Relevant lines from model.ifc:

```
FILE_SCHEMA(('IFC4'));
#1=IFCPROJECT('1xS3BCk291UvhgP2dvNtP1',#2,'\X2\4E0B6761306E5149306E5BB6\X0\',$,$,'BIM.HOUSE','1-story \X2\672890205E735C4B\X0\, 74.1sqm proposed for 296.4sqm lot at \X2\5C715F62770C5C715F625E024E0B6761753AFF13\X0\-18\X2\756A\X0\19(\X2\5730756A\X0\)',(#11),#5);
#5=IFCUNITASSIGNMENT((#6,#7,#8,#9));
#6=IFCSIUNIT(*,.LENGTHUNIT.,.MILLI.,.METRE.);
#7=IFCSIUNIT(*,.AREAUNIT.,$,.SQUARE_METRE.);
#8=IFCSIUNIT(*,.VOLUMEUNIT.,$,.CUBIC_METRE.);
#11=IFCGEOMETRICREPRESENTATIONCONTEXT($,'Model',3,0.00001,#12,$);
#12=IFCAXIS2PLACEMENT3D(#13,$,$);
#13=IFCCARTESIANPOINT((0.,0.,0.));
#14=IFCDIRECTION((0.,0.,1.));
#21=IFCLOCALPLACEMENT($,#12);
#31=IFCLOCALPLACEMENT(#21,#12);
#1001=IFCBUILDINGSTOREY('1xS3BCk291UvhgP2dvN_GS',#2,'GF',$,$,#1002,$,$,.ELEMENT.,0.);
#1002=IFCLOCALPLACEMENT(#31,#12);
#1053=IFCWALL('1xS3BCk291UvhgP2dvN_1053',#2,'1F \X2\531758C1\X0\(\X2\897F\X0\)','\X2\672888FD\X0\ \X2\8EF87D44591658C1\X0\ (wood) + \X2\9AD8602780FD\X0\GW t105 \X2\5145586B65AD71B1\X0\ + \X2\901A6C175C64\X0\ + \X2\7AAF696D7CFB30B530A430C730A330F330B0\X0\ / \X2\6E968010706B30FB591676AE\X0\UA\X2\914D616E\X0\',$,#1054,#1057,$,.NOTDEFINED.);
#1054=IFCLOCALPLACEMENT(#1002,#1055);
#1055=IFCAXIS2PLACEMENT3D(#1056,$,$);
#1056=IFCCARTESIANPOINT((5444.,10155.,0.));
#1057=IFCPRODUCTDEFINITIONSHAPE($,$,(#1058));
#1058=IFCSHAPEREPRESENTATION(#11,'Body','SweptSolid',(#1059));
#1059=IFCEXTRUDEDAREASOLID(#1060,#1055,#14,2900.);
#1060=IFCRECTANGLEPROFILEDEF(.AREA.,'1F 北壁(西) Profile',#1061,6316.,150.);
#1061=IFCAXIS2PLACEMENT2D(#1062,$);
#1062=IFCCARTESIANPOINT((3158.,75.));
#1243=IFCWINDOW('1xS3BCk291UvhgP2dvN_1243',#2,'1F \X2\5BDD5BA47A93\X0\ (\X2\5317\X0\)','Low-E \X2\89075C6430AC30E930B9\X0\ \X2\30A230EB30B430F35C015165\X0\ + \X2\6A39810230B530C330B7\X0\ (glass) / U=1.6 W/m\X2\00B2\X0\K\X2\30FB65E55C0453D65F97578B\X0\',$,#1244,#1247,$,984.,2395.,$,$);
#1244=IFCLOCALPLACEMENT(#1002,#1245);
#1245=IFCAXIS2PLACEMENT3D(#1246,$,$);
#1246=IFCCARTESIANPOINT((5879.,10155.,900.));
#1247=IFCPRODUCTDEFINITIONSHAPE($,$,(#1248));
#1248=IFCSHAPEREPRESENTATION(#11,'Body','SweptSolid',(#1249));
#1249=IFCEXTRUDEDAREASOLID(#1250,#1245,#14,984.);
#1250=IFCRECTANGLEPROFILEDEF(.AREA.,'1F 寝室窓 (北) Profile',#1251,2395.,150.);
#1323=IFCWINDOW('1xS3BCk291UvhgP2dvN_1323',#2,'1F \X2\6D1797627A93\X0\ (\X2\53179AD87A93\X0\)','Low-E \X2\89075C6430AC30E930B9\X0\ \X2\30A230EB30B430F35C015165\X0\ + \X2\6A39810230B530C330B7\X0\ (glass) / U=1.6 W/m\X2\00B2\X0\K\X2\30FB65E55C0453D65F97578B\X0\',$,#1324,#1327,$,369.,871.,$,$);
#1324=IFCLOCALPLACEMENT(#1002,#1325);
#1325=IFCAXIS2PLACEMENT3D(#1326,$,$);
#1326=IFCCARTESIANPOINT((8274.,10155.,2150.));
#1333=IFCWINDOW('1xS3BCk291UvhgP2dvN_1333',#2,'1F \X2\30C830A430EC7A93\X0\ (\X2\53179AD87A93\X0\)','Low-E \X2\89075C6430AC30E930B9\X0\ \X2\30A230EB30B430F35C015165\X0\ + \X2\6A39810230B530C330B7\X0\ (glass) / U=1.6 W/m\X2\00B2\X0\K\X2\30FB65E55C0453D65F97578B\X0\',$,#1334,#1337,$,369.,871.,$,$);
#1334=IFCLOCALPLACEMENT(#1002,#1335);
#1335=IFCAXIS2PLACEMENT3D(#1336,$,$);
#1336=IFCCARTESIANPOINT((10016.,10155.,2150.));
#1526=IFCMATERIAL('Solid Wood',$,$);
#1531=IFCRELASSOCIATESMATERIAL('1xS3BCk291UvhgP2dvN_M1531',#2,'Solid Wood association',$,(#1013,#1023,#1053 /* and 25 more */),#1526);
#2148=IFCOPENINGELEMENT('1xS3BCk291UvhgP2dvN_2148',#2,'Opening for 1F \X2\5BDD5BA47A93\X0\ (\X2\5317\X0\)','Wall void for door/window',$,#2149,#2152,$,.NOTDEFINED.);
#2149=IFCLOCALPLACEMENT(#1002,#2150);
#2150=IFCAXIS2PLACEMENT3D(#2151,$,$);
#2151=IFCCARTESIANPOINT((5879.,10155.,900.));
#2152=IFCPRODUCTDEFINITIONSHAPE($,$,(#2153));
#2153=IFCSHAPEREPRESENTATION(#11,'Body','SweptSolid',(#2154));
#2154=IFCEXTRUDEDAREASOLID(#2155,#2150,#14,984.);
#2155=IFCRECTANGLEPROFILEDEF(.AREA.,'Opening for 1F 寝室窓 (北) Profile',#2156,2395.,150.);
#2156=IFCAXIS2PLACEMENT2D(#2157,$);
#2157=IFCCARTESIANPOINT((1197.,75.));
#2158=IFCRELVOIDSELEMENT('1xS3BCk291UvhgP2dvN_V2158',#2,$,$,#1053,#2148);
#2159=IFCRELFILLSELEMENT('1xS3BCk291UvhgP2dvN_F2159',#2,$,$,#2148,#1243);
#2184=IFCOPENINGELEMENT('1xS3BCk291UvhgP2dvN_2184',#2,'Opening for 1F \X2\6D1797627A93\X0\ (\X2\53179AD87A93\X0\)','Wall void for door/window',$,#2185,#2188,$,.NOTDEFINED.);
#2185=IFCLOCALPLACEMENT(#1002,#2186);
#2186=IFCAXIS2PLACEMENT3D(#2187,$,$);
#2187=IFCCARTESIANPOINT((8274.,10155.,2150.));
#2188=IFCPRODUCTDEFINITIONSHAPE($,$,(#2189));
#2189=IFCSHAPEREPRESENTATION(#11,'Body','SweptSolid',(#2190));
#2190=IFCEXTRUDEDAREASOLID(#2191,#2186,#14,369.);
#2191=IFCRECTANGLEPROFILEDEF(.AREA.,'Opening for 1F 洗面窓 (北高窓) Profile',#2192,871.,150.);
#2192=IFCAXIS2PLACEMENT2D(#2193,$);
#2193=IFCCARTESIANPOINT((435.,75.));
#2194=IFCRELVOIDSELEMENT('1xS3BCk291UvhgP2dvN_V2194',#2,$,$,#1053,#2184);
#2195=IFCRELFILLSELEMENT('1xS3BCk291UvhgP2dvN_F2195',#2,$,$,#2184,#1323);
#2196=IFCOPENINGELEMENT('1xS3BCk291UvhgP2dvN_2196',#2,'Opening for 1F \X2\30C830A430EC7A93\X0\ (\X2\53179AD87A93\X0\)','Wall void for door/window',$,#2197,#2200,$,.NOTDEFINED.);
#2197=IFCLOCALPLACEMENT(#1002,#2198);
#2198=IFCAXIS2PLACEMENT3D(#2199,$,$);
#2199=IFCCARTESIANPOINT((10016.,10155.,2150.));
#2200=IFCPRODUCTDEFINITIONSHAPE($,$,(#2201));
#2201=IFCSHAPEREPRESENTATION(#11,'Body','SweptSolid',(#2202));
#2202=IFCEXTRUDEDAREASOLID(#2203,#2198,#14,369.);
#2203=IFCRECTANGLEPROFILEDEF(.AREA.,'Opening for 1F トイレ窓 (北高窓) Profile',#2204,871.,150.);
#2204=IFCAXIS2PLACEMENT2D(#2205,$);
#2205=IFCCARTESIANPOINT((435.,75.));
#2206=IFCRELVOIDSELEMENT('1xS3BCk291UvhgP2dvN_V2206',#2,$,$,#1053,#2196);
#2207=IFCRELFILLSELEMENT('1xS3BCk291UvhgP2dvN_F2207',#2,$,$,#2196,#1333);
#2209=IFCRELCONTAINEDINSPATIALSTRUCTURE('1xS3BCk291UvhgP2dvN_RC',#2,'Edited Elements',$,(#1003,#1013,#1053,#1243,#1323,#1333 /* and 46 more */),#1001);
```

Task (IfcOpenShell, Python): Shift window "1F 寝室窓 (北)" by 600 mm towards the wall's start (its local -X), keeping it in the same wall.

```python
import ifcopenshell
import ifcopenshell.api.geometry
import ifcopenshell.util.placement
import ifcopenshell.util.unit

model = ifcopenshell.open("model.ifc")
unit_scale = ifcopenshell.util.unit.calculate_unit_scale(model)

window = model.by_guid("1xS3BCk291UvhgP2dvN_1243")
opening = window.FillsVoids[0].RelatingOpeningElement
wall = opening.VoidsElements[0].RelatingBuildingElement

wall_matrix = ifcopenshell.util.placement.get_local_placement(wall.ObjectPlacement)
shift = wall_matrix[:3, 0] * -0.6 / unit_scale
before = ifcopenshell.util.placement.get_local_placement(window.ObjectPlacement)[:3, 3].copy()

# The window is not placed relative to its opening, so move both.
for product in (opening, window):
    matrix = ifcopenshell.util.placement.get_local_placement(product.ObjectPlacement)
    matrix[:3, 3] += shift
    ifcopenshell.api.geometry.edit_object_placement(model, product=product, matrix=matrix, is_si=False)

after = ifcopenshell.util.placement.get_local_placement(window.ObjectPlacement)[:3, 3]
print("window moved by", (after - before).round(3) + 0.0)

model.write("model_edited.ifc")
```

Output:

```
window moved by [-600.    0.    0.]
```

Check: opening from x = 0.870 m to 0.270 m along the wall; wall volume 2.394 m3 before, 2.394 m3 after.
